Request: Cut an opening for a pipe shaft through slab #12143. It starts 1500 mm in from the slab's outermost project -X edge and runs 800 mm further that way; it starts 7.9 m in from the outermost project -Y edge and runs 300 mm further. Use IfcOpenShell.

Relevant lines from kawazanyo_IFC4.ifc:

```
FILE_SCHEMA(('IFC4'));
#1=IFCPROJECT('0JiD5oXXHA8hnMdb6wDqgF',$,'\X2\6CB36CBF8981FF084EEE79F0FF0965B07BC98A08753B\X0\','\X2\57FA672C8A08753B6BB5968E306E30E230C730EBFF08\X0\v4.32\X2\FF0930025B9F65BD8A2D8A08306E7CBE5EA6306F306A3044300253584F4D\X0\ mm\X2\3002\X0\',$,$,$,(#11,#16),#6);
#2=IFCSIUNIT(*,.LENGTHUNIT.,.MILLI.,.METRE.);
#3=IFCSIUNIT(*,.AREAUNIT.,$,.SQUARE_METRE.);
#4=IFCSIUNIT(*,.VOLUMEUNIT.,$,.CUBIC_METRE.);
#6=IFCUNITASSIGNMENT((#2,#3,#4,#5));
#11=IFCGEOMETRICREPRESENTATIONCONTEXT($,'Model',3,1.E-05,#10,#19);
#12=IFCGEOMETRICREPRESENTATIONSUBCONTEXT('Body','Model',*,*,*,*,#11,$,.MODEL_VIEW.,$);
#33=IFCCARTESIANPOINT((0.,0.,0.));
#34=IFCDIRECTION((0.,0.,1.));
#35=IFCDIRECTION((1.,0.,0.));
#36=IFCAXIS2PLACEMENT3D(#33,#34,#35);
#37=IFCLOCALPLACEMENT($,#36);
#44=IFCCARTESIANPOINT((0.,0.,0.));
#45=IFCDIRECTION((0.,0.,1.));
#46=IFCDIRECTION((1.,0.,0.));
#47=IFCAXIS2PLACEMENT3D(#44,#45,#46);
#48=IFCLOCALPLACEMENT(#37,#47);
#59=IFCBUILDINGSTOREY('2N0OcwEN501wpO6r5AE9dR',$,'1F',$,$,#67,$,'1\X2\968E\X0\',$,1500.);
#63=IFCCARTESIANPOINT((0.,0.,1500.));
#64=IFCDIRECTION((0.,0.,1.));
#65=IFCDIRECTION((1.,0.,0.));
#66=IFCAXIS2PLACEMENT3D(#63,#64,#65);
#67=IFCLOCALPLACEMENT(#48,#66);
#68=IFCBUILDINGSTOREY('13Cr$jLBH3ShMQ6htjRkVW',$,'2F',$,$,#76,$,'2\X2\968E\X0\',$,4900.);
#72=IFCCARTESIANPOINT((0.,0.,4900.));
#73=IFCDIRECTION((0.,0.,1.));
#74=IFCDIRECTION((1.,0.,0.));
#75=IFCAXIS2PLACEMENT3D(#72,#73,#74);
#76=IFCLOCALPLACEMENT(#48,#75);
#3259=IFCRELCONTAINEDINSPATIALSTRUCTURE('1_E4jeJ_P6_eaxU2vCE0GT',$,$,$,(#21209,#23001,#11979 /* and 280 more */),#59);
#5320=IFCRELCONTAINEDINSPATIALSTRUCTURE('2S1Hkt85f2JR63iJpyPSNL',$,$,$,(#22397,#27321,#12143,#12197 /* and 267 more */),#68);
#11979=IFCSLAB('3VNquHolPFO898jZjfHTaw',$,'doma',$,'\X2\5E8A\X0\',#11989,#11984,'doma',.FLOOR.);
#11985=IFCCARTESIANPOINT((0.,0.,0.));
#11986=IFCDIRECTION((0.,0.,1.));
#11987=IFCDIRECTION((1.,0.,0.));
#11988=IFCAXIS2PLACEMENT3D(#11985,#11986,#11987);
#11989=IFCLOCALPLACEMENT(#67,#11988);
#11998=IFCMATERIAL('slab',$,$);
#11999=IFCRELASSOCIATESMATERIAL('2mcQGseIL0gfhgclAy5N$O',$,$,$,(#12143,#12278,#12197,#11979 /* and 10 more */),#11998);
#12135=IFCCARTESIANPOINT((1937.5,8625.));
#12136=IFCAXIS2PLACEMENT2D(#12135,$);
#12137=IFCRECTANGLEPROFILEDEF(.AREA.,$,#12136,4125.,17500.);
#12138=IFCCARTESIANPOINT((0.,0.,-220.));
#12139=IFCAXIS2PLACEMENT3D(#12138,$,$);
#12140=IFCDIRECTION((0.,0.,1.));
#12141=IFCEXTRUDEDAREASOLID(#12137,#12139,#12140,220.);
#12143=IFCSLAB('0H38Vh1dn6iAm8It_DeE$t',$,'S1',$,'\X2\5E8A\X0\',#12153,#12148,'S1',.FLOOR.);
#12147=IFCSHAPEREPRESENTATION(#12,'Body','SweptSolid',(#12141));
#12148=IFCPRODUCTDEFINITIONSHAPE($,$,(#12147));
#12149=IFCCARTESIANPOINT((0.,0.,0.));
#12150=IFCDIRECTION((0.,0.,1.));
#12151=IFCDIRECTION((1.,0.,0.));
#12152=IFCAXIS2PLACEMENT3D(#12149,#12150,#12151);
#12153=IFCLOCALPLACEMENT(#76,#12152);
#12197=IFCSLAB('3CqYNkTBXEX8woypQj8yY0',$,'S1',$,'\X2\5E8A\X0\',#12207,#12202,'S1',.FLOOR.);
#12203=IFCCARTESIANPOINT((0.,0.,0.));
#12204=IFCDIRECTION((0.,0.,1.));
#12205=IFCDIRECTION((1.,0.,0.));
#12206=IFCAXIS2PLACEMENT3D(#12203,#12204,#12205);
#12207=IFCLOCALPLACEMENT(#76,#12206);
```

```python
import numpy as np
import ifcopenshell
import ifcopenshell.api.feature
import ifcopenshell.api.geometry
import ifcopenshell.api.root
import ifcopenshell.geom
import ifcopenshell.util.placement
import ifcopenshell.util.representation
import ifcopenshell.util.shape
import ifcopenshell.util.unit

model = ifcopenshell.open("kawazanyo_IFC4.ifc")
unit_scale = ifcopenshell.util.unit.calculate_unit_scale(model)
settings = ifcopenshell.geom.settings()


def volume(element):
    """Net volume in cubic metres, openings subtracted."""
    shape = ifcopenshell.geom.create_shape(settings, element)
    return ifcopenshell.util.shape.get_volume(shape.geometry)


slab = model.by_guid("0H38Vh1dn6iAm8It_DeE$t")
before = volume(slab)

# Extent in the slab's own axes, in metres. The edges named are its -X and -Y sides.
slab_shape = ifcopenshell.geom.create_shape(settings, slab)
vertices = ifcopenshell.util.shape.get_vertices(slab_shape.geometry)
x_min, y_min, bottom = vertices.min(axis=0)
top = vertices[:, 2].max()

opening = ifcopenshell.api.root.create_entity(model, ifc_class="IfcOpeningElement", name="Pipe shaft opening", predefined_type="OPENING")
context = ifcopenshell.util.representation.get_context(model, "Model", "Body", "MODEL_VIEW")
width, depth = 0.8, 0.3
outline = [(0.0, 0.0), (width, 0.0), (width, depth), (0.0, depth), (0.0, 0.0)]
# Overshoot both faces by 50 mm so the cut is clean.
shape = ifcopenshell.api.geometry.add_slab_representation(
    model, context=context, depth=top - bottom + 0.1, polyline=outline
)
ifcopenshell.api.geometry.assign_representation(model, product=opening, representation=shape)

matrix = ifcopenshell.util.placement.get_local_placement(slab.ObjectPlacement)
matrix[:, 3] = matrix @ np.append(np.array([x_min + 1.5, y_min + 7.9, bottom - 0.05]) / unit_scale, 1.0)
ifcopenshell.api.geometry.edit_object_placement(model, product=opening, matrix=matrix, is_si=False)
ifcopenshell.api.feature.add_feature(model, feature=opening, element=slab)

after = volume(slab)

print(f"slab volume {before:.3f} -> {after:.3f} m3")

model.write("kawazanyo_IFC4_edited.ifc")
```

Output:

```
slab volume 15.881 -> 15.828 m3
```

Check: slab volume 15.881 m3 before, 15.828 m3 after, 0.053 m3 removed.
